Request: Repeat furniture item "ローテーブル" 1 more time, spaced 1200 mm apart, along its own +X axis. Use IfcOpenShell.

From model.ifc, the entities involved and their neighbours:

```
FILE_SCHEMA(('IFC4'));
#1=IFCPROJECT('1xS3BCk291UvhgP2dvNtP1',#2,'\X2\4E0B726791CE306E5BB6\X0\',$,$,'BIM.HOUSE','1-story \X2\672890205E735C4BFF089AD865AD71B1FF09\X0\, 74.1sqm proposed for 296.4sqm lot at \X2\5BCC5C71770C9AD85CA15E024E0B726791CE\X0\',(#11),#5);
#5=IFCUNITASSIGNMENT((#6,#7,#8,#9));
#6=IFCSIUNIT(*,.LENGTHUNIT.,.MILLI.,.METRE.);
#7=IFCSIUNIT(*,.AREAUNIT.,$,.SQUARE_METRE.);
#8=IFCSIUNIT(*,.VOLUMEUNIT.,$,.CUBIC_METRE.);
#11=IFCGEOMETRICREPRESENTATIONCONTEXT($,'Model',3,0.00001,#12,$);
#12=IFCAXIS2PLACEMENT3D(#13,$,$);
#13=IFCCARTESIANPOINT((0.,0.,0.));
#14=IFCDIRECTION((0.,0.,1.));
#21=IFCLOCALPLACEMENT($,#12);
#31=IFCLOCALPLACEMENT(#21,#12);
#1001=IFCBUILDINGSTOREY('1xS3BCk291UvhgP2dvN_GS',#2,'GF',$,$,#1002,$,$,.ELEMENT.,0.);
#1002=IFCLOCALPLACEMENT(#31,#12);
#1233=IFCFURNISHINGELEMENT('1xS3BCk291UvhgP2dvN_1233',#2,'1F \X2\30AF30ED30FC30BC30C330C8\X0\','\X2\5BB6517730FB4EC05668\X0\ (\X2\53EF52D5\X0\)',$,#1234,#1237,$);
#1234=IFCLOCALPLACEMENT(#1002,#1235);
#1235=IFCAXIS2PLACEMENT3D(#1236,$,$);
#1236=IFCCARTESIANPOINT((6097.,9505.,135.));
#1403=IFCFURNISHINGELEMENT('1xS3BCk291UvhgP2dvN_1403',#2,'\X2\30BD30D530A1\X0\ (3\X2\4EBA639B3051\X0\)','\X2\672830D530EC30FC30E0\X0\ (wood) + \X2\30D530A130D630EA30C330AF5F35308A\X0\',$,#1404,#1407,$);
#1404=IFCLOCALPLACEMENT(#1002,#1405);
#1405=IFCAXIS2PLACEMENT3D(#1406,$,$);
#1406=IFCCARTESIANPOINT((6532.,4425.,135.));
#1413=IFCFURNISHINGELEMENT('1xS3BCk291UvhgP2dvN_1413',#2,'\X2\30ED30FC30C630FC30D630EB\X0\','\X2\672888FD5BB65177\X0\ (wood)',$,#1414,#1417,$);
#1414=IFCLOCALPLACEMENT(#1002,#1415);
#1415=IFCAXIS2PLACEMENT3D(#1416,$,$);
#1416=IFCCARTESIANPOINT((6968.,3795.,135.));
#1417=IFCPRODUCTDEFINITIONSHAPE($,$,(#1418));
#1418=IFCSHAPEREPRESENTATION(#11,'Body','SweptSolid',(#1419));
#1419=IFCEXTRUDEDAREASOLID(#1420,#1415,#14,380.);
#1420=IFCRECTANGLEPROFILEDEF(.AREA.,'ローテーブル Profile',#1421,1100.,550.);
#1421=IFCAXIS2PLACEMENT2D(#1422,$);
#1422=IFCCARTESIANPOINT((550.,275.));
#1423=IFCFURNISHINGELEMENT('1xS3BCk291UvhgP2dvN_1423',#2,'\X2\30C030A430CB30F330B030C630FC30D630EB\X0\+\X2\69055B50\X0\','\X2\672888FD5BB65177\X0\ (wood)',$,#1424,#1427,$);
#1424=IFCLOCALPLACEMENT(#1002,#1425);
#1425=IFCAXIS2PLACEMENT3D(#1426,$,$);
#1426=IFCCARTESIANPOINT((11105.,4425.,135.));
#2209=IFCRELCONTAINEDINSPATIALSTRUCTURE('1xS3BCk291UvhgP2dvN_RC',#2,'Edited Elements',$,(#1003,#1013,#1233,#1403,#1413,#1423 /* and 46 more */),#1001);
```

```python
import ifcopenshell
import ifcopenshell.api.geometry
import ifcopenshell.api.root
import ifcopenshell.util.element
import ifcopenshell.util.placement

model = ifcopenshell.open("model.ifc")


def reuse_history(source, copy):
    """copy_class also copies each property set's owner history, people and application; keep the originals."""
    for rel in copy.IsDefinedBy:
        if rel.is_a("IfcRelDefinesByProperties") and (history := rel.RelatingPropertyDefinition.OwnerHistory):
            rel.RelatingPropertyDefinition.OwnerHistory = source.OwnerHistory
            ifcopenshell.util.element.remove_deep2(model, history)


source = model.by_guid("1xS3BCk291UvhgP2dvN_1413")
base = ifcopenshell.util.placement.get_local_placement(source.ObjectPlacement)
step = base[:3, 0] * 1200.0

for i in range(1, 2):
    copy = ifcopenshell.api.root.copy_class(model, product=source)
    copy.Representation = ifcopenshell.util.element.copy_deep(
        model, source.Representation, exclude=["IfcGeometricRepresentationContext", "IfcRepresentationMap"]
    )
    reuse_history(source, copy)
    matrix = base.copy()
    matrix[:3, 3] += i * step
    print("added at", matrix[:3, 3].round(3) + 0.0)
    ifcopenshell.api.geometry.edit_object_placement(model, product=copy, matrix=matrix, is_si=False)

model.write("model-out.ifc")
```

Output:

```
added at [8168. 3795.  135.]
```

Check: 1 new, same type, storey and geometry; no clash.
